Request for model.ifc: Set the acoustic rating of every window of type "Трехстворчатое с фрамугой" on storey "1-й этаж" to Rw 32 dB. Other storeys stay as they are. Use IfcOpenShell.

First a look at what the model holds.

```python
import ifcopenshell
import ifcopenshell.util.element

model = ifcopenshell.open("model.ifc")
print(model.schema)
storey = next(s for s in model.by_type("IfcBuildingStorey") if s.Name == "1-й этаж")
windows = [e for e in ifcopenshell.util.element.get_decomposition(storey) if e.is_a("IfcWindow")]
seen = {}
for e in windows:
    element_type = ifcopenshell.util.element.get_type(e)
    key = (element_type.Name if element_type != e and element_type else None, ifcopenshell.util.element.get_pset(e, "Pset_WindowCommon", "AcousticRating"))
    seen[key] = seen.get(key, 0) + 1
for (name, value), count in sorted(seen.items(), key=str):
    print(count, "x", name, "|", value)
```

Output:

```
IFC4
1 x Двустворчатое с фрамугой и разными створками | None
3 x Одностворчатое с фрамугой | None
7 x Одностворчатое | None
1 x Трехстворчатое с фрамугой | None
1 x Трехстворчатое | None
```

```python
import ifcopenshell
import ifcopenshell.api.pset
import ifcopenshell.util.element

model = ifcopenshell.open("model.ifc")

storey = next(s for s in model.by_type("IfcBuildingStorey") if s.Name == "1-й этаж")
windows = [e for e in ifcopenshell.util.element.get_decomposition(storey) if e.is_a("IfcWindow")]

count = 0
for e in windows:
    element_type = ifcopenshell.util.element.get_type(e)
    if element_type in (None, e) or element_type.Name != "Трехстворчатое с фрамугой":
        continue
    # add_pset returns the element's existing set when there is one.
    pset = ifcopenshell.api.pset.add_pset(model, product=e, name="Pset_WindowCommon")
    ifcopenshell.api.pset.edit_pset(model, pset=pset, properties={"AcousticRating": "Rw 32 dB"})
    count += 1

print(count, "windows updated")

model.write("model_rev.ifc")
```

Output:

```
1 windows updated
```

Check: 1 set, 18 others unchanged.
